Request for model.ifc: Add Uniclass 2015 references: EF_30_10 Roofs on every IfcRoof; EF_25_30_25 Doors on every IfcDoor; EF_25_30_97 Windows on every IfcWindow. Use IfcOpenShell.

First a look at what the model holds.

```python
import ifcopenshell

model = ifcopenshell.open("model.ifc")
print(model.schema)
print("classifications:", [c.Name for c in model.by_type("IfcClassification")])
for ifc_class in ("IfcDoor", "IfcRoof", "IfcStair", "IfcWall", "IfcWindow"):
    print(ifc_class, len(model.by_type(ifc_class)))
```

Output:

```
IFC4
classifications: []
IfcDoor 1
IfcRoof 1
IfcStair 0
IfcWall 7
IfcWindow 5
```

```python
import ifcopenshell
import ifcopenshell.api.classification

model = ifcopenshell.open("model.ifc")

system = ifcopenshell.api.classification.add_classification(model, classification="Uniclass 2015")

codes = {
    "IfcRoof": ("EF_30_10", "Roofs"),
    "IfcDoor": ("EF_25_30_25", "Doors"),
    "IfcWindow": ("EF_25_30_97", "Windows"),
}
for ifc_class, (code, name) in codes.items():
    products = model.by_type(ifc_class)
    ifcopenshell.api.classification.add_reference(
        model, products=products, classification=system, identification=code, name=name
    )
    print(code, len(products))

model.write("model_edited.ifc")
```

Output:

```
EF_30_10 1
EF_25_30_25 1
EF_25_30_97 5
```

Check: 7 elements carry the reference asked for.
